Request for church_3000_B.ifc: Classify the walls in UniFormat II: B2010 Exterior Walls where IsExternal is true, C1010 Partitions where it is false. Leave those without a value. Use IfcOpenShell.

First a look at what the model holds.

```python
import ifcopenshell
import ifcopenshell.util.element

model = ifcopenshell.open("church_3000_B.ifc")
print(model.schema)
print("classifications:", [c.Name for c in model.by_type("IfcClassification")])
values = [ifcopenshell.util.element.get_pset(e, "Pset_WallCommon", "IsExternal") for e in model.by_type("IfcWall")]
for value in (True, False, None):
    print("IsExternal", value, values.count(value))
```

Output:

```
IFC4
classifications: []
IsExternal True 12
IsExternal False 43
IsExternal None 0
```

```python
import ifcopenshell
import ifcopenshell.api.classification
import ifcopenshell.util.element

model = ifcopenshell.open("church_3000_B.ifc")

system = ifcopenshell.api.classification.add_classification(model, classification="UniFormat II")

walls = model.by_type("IfcWall")
external = {e: ifcopenshell.util.element.get_pset(e, "Pset_WallCommon", "IsExternal") for e in walls}
for flag, code, name in ((True, "B2010", "Exterior Walls"), (False, "C1010", "Partitions")):
    products = [e for e in walls if external[e] is flag]
    ifcopenshell.api.classification.add_reference(
        model, products=products, classification=system, identification=code, name=name
    )
    print(code, len(products))

model.write("church_3000_B_v2.ifc")
```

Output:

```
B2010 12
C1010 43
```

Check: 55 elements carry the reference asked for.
